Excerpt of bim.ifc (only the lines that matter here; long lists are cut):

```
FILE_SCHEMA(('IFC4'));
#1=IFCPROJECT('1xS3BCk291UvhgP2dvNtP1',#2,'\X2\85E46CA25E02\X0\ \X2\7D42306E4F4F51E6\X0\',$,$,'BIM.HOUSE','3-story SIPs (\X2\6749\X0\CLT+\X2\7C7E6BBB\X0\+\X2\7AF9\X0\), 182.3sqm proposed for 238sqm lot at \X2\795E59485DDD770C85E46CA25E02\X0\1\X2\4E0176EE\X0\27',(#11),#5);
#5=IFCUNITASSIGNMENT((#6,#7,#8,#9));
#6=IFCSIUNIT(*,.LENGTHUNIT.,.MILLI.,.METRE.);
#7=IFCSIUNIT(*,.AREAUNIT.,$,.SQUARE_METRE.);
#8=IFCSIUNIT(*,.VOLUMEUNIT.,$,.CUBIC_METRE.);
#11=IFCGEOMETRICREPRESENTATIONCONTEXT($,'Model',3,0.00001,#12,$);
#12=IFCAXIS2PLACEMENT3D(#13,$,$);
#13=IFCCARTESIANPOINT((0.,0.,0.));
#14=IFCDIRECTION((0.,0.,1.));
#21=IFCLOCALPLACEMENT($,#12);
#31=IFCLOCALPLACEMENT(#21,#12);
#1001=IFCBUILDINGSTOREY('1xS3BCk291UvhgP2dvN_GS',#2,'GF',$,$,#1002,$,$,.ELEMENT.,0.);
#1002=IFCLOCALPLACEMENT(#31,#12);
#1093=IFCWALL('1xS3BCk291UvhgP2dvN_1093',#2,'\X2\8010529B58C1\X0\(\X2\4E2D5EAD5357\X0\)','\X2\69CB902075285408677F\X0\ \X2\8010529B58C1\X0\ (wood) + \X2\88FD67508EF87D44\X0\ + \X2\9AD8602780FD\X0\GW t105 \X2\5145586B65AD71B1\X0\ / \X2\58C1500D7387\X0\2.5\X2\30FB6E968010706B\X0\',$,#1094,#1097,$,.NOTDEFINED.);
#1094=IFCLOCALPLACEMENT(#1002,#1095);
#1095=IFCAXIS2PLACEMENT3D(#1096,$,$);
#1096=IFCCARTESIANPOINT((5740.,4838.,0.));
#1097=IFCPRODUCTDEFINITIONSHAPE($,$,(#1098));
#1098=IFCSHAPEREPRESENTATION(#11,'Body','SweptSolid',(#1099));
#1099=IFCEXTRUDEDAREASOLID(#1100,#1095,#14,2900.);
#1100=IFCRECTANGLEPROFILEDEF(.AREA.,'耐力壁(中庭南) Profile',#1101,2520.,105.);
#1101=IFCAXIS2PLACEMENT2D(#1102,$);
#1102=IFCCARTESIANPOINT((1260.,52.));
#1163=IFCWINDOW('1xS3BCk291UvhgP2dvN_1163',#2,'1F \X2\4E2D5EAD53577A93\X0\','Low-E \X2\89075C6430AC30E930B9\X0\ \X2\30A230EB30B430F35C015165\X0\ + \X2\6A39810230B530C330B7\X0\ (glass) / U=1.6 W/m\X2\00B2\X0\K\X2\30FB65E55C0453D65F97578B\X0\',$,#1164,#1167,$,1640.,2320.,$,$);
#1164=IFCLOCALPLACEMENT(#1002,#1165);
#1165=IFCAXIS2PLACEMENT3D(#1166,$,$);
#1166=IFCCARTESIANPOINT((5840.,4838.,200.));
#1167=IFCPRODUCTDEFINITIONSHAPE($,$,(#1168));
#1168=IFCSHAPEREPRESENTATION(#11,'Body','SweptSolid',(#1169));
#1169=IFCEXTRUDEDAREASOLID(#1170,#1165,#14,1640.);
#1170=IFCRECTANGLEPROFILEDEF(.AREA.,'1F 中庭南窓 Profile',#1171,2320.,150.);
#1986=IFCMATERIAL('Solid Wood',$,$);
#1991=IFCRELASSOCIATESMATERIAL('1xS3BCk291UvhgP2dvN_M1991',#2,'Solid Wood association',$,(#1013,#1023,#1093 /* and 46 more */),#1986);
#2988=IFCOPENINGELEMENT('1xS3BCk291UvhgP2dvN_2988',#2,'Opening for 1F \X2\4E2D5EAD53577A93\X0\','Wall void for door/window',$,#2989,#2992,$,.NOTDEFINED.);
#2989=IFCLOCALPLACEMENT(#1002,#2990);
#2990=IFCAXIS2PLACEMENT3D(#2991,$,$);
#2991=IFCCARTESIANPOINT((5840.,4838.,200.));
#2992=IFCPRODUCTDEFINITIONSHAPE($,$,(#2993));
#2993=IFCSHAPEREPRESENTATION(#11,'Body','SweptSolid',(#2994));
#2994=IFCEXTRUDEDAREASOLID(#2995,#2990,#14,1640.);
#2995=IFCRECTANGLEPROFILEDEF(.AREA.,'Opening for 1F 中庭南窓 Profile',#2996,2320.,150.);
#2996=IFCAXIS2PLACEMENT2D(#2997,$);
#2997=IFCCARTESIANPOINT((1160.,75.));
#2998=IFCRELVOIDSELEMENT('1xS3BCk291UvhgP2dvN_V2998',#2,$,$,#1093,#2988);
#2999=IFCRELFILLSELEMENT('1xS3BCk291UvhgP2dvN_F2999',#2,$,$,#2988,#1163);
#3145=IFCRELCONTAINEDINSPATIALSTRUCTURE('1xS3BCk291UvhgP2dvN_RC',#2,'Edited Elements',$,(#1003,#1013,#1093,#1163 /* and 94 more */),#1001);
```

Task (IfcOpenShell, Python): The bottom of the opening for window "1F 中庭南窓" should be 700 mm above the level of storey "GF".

```python
import numpy as np
import ifcopenshell
import ifcopenshell.api.geometry
import ifcopenshell.geom
import ifcopenshell.util.element
import ifcopenshell.util.placement
import ifcopenshell.util.shape
import ifcopenshell.util.unit

model = ifcopenshell.open("bim.ifc")
unit_scale = ifcopenshell.util.unit.calculate_unit_scale(model)

window = model.by_guid("1xS3BCk291UvhgP2dvN_1163")
opening = window.FillsVoids[0].RelatingOpeningElement
storey = ifcopenshell.util.element.get_container(window, ifc_class="IfcBuildingStorey")
level = ifcopenshell.util.placement.get_local_placement(storey.ObjectPlacement)[2, 3]

# The opening's origin need not be at the sill, so measure its lowest point.
shape = ifcopenshell.geom.create_shape(ifcopenshell.geom.settings(), opening)
bottom = ifcopenshell.util.shape.get_shape_bottom_elevation(shape, shape.geometry) / unit_scale
dz = level + 0.7 / unit_scale - bottom

shift = np.array([0.0, 0.0, dz])
# The window is not placed relative to its opening, so move both.
for product in (opening, window):
    matrix = ifcopenshell.util.placement.get_local_placement(product.ObjectPlacement)
    matrix[:3, 3] += shift
    ifcopenshell.api.geometry.edit_object_placement(model, product=product, matrix=matrix, is_si=False)

print(f"moved by {dz * unit_scale:+.3f} m")

model.write("bim-out.ifc")
```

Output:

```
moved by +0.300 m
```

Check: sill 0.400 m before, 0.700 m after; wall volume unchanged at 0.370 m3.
